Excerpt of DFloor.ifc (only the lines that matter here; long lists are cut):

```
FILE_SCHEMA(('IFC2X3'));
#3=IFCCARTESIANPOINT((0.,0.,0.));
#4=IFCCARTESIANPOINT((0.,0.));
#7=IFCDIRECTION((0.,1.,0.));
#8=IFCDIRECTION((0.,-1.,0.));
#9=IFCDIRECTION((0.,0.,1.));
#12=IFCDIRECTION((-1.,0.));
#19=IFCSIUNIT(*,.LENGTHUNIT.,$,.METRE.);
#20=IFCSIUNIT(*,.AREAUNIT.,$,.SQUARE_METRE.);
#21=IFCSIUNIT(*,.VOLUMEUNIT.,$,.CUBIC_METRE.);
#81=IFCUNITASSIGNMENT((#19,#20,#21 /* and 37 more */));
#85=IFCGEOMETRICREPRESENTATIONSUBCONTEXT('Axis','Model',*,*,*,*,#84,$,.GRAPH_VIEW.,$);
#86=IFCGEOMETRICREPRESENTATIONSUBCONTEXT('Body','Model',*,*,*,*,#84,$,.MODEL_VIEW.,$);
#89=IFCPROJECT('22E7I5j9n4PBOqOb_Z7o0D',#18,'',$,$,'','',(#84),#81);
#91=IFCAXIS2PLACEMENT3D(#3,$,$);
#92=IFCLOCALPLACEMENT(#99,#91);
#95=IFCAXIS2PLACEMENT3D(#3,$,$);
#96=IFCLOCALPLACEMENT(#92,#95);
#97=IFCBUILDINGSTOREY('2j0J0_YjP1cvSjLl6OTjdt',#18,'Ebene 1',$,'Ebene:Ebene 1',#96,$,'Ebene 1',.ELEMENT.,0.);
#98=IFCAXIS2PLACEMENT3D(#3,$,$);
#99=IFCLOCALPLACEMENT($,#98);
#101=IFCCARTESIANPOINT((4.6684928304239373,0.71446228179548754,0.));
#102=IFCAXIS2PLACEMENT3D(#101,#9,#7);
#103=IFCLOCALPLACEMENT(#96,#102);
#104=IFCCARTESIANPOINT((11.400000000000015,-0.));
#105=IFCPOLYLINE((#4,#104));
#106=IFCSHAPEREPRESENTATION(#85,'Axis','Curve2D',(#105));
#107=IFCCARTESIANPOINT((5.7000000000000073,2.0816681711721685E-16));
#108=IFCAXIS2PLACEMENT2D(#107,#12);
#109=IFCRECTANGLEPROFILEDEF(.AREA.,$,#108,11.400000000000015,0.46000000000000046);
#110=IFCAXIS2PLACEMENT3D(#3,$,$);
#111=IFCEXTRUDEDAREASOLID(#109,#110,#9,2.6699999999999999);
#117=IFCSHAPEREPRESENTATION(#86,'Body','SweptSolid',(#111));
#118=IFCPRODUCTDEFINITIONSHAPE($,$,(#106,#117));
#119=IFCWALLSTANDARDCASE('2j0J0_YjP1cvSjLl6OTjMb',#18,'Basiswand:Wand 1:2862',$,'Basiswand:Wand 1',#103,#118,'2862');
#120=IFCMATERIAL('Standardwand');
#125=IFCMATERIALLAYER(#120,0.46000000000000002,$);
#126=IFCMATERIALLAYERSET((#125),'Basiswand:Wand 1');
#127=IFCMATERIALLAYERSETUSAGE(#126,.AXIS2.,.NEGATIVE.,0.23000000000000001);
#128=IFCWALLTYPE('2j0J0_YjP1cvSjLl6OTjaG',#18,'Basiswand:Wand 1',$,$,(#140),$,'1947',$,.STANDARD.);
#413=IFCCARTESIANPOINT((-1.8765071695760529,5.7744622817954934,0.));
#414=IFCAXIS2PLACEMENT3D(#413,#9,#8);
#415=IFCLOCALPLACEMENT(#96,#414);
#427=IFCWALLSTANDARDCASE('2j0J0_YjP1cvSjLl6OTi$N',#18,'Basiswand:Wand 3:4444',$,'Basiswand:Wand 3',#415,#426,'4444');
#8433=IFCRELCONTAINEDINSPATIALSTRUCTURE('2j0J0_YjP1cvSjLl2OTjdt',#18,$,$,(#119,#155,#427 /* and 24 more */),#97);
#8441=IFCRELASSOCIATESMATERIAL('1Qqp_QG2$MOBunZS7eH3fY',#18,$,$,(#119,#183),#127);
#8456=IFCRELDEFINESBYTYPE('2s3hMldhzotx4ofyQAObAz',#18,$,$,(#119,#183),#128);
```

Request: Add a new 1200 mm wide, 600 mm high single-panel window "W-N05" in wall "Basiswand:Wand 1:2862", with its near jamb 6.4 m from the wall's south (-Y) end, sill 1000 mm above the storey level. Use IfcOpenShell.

```python
import numpy as np
import ifcopenshell
import ifcopenshell.api.feature
import ifcopenshell.api.geometry
import ifcopenshell.api.root
import ifcopenshell.api.spatial
import ifcopenshell.api.type
import ifcopenshell.geom
import ifcopenshell.util.element
import ifcopenshell.util.placement
import ifcopenshell.util.representation
import ifcopenshell.util.shape
import ifcopenshell.util.unit

model = ifcopenshell.open("DFloor.ifc")
unit_scale = ifcopenshell.util.unit.calculate_unit_scale(model)
settings = ifcopenshell.geom.settings()


def volume(element):
    """Net volume in cubic metres, openings subtracted."""
    shape = ifcopenshell.geom.create_shape(settings, element)
    return ifcopenshell.util.shape.get_volume(shape.geometry)


wall = model.by_guid("2j0J0_YjP1cvSjLl6OTjMb")
storey = ifcopenshell.util.element.get_container(wall, ifc_class="IfcBuildingStorey")
context = ifcopenshell.util.representation.get_context(model, "Model", "Body", "MODEL_VIEW")
before = volume(wall)

width, height, from_end, sill = 1.2, 0.6, 6.4, 1  # metres

# The wall runs along its own X axis, and the end named is its -X end.
wall_shape = ifcopenshell.geom.create_shape(settings, wall)
x, y, z = ifcopenshell.util.shape.get_vertices(wall_shape.geometry).T
start = x.min() + from_end
face, thickness = float(y.min()), float(y.max() - y.min())
wall_matrix = ifcopenshell.util.placement.get_local_placement(wall.ObjectPlacement)
level = ifcopenshell.util.placement.get_local_placement(storey.ObjectPlacement)[2, 3]


def in_wall(x, y):
    """Placement at x, y metres in the wall's axes, at sill height."""
    matrix = wall_matrix.copy()
    matrix[:, 3] = wall_matrix @ np.array([x / unit_scale, y / unit_scale, 0.0, 1.0])
    matrix[2, 3] = level + sill / unit_scale
    return matrix


# Opening: a box that overshoots both wall faces by 50 mm.
opening = ifcopenshell.api.root.create_entity(model, ifc_class="IfcOpeningElement")
box = ifcopenshell.api.geometry.add_wall_representation(
    model, context=context, length=width, height=height, thickness=thickness + 0.1
)
ifcopenshell.api.geometry.assign_representation(model, product=opening, representation=box)
ifcopenshell.api.geometry.edit_object_placement(model, product=opening, matrix=in_wall(start, face - 0.05), is_si=False)
ifcopenshell.api.feature.add_feature(model, feature=opening, element=wall)

window = ifcopenshell.api.root.create_entity(model, ifc_class="IfcWindow", name="W-N05")
window.OverallWidth, window.OverallHeight = width / unit_scale, height / unit_scale
body = ifcopenshell.api.geometry.add_window_representation(
    model,
    context=context,
    overall_width=window.OverallWidth,
    overall_height=window.OverallHeight,
    partition_type="SINGLE_PANEL",
)
ifcopenshell.api.geometry.assign_representation(model, product=window, representation=body)
ifcopenshell.api.spatial.assign_container(model, products=[window], relating_structure=storey)
fills = ifcopenshell.api.feature.add_filling(model, opening=opening, element=window)
fills.OwnerHistory = window.OwnerHistory  # required in IFC2X3

# IFC2X3 keeps the operation on the window style.
style = ifcopenshell.api.root.create_entity(model, ifc_class="IfcWindowStyle", name="W-N05")
style.OperationType, style.ConstructionType = "SINGLE_PANEL", "NOTDEFINED"
style.ParameterTakesPrecedence = style.Sizeable = False
ifcopenshell.api.type.assign_type(model, related_objects=[window], relating_type=style)

# Centre the window in the wall's thickness.
ifcopenshell.api.geometry.edit_object_placement(model, product=window, matrix=in_wall(start, face), is_si=False)
window_shape = ifcopenshell.geom.create_shape(settings, window)
depth = ifcopenshell.util.shape.get_vertices(window_shape.geometry)[:, 1]
offset = face + thickness / 2 - (depth.min() + depth.max()) / 2
ifcopenshell.api.geometry.edit_object_placement(model, product=window, matrix=in_wall(start, offset), is_si=False)

after = volume(wall)

print(f"wall volume {before:.3f} -> {after:.3f} m3")

model.write("DFloor-out.ifc")
```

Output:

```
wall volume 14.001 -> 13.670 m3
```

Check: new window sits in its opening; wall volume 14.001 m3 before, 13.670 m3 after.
